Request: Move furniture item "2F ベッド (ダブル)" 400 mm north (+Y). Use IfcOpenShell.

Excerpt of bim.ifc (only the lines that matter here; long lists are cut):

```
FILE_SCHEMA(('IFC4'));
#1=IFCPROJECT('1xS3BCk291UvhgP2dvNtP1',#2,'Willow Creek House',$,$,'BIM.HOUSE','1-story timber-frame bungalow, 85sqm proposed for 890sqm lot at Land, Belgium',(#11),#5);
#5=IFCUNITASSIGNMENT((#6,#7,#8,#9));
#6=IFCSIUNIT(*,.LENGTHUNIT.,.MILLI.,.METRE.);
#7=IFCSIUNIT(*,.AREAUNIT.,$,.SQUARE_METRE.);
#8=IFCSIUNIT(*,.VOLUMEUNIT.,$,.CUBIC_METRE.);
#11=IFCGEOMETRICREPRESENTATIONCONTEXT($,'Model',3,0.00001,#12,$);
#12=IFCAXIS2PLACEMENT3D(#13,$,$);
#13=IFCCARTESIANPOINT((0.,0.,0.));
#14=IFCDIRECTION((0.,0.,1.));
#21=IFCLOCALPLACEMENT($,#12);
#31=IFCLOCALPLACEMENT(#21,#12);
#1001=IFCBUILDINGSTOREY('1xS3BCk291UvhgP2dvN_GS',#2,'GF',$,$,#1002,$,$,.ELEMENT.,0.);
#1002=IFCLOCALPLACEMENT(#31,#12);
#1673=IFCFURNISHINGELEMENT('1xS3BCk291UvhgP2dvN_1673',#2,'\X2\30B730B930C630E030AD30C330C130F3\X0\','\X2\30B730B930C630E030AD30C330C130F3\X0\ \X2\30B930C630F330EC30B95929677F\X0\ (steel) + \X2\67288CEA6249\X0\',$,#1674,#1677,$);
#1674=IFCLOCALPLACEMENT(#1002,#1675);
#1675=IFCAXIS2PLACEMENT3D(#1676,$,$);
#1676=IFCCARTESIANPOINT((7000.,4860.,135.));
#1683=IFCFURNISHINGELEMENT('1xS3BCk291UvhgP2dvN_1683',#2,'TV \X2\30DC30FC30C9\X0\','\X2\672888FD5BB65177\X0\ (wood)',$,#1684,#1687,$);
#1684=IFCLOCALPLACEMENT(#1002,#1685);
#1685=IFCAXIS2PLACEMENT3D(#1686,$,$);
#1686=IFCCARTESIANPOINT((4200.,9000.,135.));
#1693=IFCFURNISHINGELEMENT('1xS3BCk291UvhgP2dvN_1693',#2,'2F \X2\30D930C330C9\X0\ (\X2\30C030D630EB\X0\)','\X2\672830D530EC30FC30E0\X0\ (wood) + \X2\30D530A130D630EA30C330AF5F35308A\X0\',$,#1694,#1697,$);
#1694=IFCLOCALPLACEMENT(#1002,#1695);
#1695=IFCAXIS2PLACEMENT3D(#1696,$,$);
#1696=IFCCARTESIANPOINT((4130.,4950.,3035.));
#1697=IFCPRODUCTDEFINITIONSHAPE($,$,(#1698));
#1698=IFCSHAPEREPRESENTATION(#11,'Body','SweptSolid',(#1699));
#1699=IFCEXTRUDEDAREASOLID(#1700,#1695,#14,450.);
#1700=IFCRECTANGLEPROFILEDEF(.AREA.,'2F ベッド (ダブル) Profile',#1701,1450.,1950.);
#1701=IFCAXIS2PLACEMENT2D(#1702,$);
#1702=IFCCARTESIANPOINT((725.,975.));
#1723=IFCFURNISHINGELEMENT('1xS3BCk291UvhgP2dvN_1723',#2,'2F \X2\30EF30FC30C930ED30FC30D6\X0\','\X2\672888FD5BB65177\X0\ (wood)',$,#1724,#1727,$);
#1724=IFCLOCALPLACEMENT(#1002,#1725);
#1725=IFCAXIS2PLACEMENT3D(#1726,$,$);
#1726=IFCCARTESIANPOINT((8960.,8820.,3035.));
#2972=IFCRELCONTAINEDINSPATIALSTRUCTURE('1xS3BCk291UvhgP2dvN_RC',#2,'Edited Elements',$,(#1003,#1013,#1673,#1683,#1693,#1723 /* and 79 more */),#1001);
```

```python
import ifcopenshell
import ifcopenshell.api.geometry
import ifcopenshell.util.placement
import ifcopenshell.util.unit

model = ifcopenshell.open("bim.ifc")
unit_scale = ifcopenshell.util.unit.calculate_unit_scale(model)

item = model.by_id(1693)
matrix = ifcopenshell.util.placement.get_local_placement(item.ObjectPlacement)
matrix[1, 3] += 0.4 / unit_scale
ifcopenshell.api.geometry.edit_object_placement(model, product=item, matrix=matrix, is_si=False)

print(ifcopenshell.util.placement.get_local_placement(item.ObjectPlacement).round(3) + 0.0)

model.write("bim_rev.ifc")
```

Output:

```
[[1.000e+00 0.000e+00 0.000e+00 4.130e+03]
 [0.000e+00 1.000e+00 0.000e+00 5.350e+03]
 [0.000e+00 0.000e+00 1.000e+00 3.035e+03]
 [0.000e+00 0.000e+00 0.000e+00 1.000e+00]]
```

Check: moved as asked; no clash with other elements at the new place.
